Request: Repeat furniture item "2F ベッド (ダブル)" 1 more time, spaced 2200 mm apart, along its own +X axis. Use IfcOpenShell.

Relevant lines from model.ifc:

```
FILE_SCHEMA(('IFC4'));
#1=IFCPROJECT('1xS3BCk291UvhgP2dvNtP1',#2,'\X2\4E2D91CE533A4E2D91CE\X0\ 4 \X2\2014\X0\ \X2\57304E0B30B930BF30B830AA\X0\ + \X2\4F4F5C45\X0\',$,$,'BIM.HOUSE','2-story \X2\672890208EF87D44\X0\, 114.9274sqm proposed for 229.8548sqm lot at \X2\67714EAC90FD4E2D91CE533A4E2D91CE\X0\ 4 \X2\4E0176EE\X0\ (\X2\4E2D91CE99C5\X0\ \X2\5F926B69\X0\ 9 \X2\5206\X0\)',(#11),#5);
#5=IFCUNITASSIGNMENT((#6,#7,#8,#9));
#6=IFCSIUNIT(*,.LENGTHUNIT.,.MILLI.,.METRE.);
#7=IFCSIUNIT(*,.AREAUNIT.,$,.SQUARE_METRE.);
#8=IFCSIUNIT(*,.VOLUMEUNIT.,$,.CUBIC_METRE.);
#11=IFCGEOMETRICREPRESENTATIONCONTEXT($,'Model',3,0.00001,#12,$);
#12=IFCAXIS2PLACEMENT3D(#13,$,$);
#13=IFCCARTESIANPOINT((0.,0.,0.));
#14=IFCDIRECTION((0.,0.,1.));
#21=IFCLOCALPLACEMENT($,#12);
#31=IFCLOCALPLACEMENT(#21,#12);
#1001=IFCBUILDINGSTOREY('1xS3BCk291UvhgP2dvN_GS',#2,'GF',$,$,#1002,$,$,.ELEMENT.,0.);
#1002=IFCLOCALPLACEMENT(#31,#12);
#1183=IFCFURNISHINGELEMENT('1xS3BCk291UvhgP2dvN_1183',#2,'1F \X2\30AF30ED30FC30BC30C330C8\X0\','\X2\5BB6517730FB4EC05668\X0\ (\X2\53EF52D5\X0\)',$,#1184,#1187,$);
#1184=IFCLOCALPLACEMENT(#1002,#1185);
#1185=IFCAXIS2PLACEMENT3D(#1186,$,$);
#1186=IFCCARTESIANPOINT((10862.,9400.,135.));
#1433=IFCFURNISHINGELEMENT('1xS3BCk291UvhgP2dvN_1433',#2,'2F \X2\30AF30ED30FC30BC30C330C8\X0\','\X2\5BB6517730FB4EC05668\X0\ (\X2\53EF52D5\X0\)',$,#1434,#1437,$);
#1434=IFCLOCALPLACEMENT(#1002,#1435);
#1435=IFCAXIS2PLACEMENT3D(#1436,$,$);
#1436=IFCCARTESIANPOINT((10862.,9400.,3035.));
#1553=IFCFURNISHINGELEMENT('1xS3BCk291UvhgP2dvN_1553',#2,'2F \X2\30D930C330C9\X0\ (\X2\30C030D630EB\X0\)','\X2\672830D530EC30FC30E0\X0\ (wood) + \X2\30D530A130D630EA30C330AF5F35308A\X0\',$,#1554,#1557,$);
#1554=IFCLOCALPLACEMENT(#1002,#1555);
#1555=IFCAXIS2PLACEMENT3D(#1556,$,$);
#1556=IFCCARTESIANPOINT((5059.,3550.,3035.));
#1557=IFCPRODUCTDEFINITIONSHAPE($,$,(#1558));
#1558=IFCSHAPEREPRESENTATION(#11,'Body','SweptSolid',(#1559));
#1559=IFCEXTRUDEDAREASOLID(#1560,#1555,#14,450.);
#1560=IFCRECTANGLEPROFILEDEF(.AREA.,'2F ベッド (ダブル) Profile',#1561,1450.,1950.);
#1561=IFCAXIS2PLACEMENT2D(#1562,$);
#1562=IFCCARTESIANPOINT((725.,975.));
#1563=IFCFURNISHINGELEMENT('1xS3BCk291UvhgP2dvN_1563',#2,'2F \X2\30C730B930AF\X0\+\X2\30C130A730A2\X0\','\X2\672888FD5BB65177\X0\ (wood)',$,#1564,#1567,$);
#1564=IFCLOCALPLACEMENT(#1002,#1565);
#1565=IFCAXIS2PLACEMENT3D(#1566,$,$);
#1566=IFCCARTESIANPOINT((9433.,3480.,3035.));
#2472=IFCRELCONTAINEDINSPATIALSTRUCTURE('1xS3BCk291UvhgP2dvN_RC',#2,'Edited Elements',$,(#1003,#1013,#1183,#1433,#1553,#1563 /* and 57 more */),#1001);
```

```python
import ifcopenshell
import ifcopenshell.api.geometry
import ifcopenshell.api.root
import ifcopenshell.util.element
import ifcopenshell.util.placement
import ifcopenshell.util.unit

model = ifcopenshell.open("model.ifc")
unit_scale = ifcopenshell.util.unit.calculate_unit_scale(model)


def reuse_history(source, copy):
    """copy_class also copies each property set's owner history, people and application; keep the originals."""
    for rel in copy.IsDefinedBy:
        if rel.is_a("IfcRelDefinesByProperties") and (history := rel.RelatingPropertyDefinition.OwnerHistory):
            rel.RelatingPropertyDefinition.OwnerHistory = source.OwnerHistory
            ifcopenshell.util.element.remove_deep2(model, history)


source = model.by_guid("1xS3BCk291UvhgP2dvN_1553")
base = ifcopenshell.util.placement.get_local_placement(source.ObjectPlacement)
step = base[:3, 0] * 2.2 / unit_scale

for i in range(1, 2):
    copy = ifcopenshell.api.root.copy_class(model, product=source)
    copy.Representation = ifcopenshell.util.element.copy_deep(
        model, source.Representation, exclude=["IfcGeometricRepresentationContext", "IfcRepresentationMap"]
    )
    reuse_history(source, copy)
    matrix = base.copy()
    matrix[:3, 3] += i * step
    print("added at", matrix[:3, 3].round(3) + 0.0)
    ifcopenshell.api.geometry.edit_object_placement(model, product=copy, matrix=matrix, is_si=False)

model.write("model_rev.ifc")
```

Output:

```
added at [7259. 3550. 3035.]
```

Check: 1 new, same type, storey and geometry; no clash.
